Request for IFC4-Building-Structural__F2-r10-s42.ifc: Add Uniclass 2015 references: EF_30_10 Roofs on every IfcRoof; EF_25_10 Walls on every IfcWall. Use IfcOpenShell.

First a look at what the model holds.

```python
import ifcopenshell

model = ifcopenshell.open("IFC4-Building-Structural__F2-r10-s42.ifc")
print(model.schema)
print("classifications:", [c.Name for c in model.by_type("IfcClassification")])
for ifc_class in ("IfcDoor", "IfcRoof", "IfcStair", "IfcWall", "IfcWindow"):
    print(ifc_class, len(model.by_type(ifc_class)))
```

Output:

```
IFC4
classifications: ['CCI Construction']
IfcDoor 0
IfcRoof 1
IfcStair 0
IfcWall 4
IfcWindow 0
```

```python
import ifcopenshell
import ifcopenshell.api.classification

model = ifcopenshell.open("IFC4-Building-Structural__F2-r10-s42.ifc")

system = ifcopenshell.api.classification.add_classification(model, classification="Uniclass 2015")

codes = {
    "IfcRoof": ("EF_30_10", "Roofs"),
    "IfcWall": ("EF_25_10", "Walls"),
}
for ifc_class, (code, name) in codes.items():
    products = model.by_type(ifc_class)
    ifcopenshell.api.classification.add_reference(
        model, products=products, classification=system, identification=code, name=name
    )
    print(code, len(products))

model.write("IFC4-Building-Structural__F2-r10-s42_edited.ifc")
```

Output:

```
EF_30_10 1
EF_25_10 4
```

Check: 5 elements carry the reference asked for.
